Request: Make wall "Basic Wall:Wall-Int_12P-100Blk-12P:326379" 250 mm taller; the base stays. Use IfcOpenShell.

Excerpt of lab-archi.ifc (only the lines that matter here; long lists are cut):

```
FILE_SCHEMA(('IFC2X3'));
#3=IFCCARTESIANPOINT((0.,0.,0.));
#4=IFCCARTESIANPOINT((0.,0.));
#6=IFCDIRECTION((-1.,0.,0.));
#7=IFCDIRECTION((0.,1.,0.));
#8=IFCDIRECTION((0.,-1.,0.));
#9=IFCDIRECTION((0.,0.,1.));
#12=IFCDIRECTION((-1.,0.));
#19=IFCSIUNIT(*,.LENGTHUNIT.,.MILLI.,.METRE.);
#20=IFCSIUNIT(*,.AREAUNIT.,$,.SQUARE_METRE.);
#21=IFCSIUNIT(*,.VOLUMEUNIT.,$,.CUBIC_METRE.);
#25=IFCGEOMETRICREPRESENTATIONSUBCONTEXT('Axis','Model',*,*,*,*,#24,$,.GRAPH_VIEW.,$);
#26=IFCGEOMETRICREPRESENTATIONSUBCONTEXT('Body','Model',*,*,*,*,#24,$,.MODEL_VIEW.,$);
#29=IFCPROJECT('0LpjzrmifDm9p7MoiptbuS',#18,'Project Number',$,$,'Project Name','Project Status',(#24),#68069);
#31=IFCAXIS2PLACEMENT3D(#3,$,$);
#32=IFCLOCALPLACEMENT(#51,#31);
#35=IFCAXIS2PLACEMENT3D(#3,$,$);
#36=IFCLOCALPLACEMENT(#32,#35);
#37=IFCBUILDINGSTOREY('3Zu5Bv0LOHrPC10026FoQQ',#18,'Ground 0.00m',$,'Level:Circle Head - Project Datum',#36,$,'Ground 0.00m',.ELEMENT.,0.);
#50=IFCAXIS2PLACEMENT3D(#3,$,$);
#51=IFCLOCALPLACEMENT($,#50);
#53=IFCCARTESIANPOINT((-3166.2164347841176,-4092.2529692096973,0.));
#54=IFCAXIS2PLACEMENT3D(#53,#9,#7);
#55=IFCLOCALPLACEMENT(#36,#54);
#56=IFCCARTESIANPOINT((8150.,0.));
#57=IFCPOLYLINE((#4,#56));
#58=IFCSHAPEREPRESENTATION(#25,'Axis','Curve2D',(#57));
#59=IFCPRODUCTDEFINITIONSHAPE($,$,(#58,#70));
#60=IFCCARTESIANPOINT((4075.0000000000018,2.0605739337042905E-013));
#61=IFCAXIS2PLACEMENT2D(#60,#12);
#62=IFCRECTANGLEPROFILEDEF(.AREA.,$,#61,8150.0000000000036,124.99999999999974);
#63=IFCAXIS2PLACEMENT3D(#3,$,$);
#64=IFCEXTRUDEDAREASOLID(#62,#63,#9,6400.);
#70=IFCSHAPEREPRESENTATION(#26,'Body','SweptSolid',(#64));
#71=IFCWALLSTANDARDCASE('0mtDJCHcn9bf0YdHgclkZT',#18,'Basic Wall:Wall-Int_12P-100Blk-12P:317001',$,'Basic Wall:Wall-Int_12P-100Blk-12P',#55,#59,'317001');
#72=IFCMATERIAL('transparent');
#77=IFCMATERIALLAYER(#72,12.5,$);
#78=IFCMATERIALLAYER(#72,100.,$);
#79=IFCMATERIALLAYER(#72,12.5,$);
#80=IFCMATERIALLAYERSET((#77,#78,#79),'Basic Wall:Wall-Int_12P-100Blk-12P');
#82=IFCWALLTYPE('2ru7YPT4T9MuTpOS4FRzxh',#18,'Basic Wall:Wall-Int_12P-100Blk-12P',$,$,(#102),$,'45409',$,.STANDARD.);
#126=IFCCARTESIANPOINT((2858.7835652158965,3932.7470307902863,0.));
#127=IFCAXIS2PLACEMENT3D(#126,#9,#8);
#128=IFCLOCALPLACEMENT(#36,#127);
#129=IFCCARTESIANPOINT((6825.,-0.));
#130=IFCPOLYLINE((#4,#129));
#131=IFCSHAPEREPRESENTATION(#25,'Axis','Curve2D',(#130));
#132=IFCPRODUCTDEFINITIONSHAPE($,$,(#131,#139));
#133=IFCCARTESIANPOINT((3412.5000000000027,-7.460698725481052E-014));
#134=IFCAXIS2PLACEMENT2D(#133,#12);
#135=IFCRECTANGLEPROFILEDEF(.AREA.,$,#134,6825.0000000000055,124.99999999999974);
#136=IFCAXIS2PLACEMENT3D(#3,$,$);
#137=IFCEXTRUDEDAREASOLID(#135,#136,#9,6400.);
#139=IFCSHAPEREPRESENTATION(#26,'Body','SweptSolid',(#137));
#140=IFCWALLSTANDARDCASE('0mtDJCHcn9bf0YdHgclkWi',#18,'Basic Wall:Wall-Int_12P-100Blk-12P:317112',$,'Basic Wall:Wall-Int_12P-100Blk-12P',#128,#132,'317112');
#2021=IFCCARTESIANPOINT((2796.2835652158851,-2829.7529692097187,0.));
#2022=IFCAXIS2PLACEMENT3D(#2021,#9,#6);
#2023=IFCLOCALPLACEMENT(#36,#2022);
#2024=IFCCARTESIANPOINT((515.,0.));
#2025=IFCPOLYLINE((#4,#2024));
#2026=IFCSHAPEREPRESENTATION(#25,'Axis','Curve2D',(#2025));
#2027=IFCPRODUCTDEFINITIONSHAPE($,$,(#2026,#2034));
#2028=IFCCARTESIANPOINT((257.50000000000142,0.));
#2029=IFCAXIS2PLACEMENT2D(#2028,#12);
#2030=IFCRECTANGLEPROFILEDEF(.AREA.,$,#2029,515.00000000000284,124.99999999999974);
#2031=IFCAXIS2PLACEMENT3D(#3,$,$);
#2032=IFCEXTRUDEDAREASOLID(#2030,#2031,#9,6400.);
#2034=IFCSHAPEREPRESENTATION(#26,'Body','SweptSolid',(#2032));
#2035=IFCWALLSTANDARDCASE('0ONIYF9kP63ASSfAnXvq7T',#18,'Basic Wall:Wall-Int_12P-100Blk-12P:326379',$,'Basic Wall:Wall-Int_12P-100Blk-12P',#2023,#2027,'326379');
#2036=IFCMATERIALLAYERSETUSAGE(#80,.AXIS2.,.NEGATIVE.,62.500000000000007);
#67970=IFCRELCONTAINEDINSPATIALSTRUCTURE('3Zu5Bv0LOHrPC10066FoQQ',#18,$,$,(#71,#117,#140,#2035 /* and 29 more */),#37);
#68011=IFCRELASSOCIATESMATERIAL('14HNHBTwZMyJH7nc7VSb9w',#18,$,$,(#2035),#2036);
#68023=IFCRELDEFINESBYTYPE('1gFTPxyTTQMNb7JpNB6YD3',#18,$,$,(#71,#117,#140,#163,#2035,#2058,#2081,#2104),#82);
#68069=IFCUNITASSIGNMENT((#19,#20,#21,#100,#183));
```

```python
import ifcopenshell
import ifcopenshell.geom
import ifcopenshell.util.representation
import ifcopenshell.util.shape
import ifcopenshell.util.unit

model = ifcopenshell.open("lab-archi.ifc")
unit_scale = ifcopenshell.util.unit.calculate_unit_scale(model)
settings = ifcopenshell.geom.settings()


def volume(element):
    """Net volume in cubic metres, openings subtracted."""
    shape = ifcopenshell.geom.create_shape(settings, element)
    return ifcopenshell.util.shape.get_volume(shape.geometry)


wall = model.by_guid("0ONIYF9kP63ASSfAnXvq7T")
before = volume(wall)

body = ifcopenshell.util.representation.get_representation(wall, "Model", "Body")
solid = body.Items[0]
old_height = solid.Depth
solid.Depth += 0.25 / unit_scale
after = volume(wall)

print(f"height {old_height:g} -> {solid.Depth:g}, volume {before:.3f} -> {after:.3f} m3")

model.write("lab-archi-out.ifc")
```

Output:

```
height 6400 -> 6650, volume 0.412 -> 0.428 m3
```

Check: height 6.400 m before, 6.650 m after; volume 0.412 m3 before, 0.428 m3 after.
